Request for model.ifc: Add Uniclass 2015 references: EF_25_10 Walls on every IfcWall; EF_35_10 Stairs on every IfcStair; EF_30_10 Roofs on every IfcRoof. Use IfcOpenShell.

First a look at what the model holds.

```python
import ifcopenshell

model = ifcopenshell.open("model.ifc")
print(model.schema)
print("classifications:", [c.Name for c in model.by_type("IfcClassification")])
for ifc_class in ("IfcDoor", "IfcRoof", "IfcStair", "IfcWall", "IfcWindow"):
    print(ifc_class, len(model.by_type(ifc_class)))
```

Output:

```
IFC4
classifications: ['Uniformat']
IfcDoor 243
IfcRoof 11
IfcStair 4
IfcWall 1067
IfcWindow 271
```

```python
import ifcopenshell
import ifcopenshell.api.classification

model = ifcopenshell.open("model.ifc")

system = ifcopenshell.api.classification.add_classification(model, classification="Uniclass 2015")

codes = {
    "IfcWall": ("EF_25_10", "Walls"),
    "IfcStair": ("EF_35_10", "Stairs"),
    "IfcRoof": ("EF_30_10", "Roofs"),
}
for ifc_class, (code, name) in codes.items():
    products = model.by_type(ifc_class)
    ifcopenshell.api.classification.add_reference(
        model, products=products, classification=system, identification=code, name=name
    )
    print(code, len(products))

model.write("model_updated.ifc")
```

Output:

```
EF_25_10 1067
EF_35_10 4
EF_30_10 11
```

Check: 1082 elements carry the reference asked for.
